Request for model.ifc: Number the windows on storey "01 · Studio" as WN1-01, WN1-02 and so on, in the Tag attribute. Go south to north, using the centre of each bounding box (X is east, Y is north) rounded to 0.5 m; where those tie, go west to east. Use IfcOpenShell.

First a look at what the model holds.

```python
import ifcopenshell
import ifcopenshell.util.element
import ifcopenshell.util.placement

model = ifcopenshell.open("model.ifc")
print(model.schema)
storey = next(s for s in model.by_type("IfcBuildingStorey") if s.Name == "01 · Studio")
windows = [e for e in ifcopenshell.util.element.get_decomposition(storey) if e.is_a("IfcWindow")]
for e in sorted(windows, key=lambda e: e.id()):
    origin = ifcopenshell.util.placement.get_local_placement(e.ObjectPlacement)[:3, 3]
    print(e.id(), e.Tag, e.Name, origin.round(2) + 0.0, sep=" | ")
```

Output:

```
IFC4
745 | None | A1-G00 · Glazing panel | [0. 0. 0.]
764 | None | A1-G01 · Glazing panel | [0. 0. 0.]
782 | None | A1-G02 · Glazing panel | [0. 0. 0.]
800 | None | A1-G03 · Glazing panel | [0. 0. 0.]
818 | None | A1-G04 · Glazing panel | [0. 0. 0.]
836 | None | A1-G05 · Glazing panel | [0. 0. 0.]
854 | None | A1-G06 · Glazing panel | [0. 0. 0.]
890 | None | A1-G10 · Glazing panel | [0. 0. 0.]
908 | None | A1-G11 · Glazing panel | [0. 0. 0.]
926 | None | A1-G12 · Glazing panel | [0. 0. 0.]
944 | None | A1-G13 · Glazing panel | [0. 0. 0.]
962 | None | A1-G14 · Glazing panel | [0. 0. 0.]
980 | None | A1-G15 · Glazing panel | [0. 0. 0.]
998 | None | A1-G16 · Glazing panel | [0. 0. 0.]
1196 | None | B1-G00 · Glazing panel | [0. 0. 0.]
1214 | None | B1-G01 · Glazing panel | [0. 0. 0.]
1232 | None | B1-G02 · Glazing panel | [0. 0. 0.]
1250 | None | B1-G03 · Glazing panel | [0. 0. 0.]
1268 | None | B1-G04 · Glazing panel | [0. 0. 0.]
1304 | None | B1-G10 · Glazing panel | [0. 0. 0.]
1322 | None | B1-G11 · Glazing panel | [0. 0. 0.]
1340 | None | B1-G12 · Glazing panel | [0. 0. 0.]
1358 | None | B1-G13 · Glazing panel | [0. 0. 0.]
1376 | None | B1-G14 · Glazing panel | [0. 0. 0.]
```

```python
import ifcopenshell
import ifcopenshell.geom
import ifcopenshell.util.element
import ifcopenshell.util.shape

model = ifcopenshell.open("model.ifc")
settings = ifcopenshell.geom.settings()
settings.set("use-world-coords", True)


def centre(element):
    shape = ifcopenshell.geom.create_shape(settings, element)
    return ifcopenshell.util.shape.get_bbox_centroid(shape.geometry)


storey = next(s for s in model.by_type("IfcBuildingStorey") if s.Name == "01 · Studio")
windows = [e for e in ifcopenshell.util.element.get_decomposition(storey) if e.is_a("IfcWindow")]

# Insertion points can sit at a corner or the storey origin, so sort by the geometry (in metres).
centres = {e: centre(e) for e in windows}
windows.sort(key=lambda e: (round(centres[e][1] / 0.5), centres[e][0]))

for i, e in enumerate(windows, start=1):
    number = f"WN1-{i:02d}"
    e.Tag = number
    print(e.id(), number)

model.write("model_v2.ifc")
```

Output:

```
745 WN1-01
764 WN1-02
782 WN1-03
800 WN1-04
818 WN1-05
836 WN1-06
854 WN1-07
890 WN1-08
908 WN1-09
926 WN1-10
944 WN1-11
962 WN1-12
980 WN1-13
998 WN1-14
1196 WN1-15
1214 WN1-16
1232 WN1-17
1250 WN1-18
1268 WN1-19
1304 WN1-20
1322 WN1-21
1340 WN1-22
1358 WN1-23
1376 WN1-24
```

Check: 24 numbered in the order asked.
